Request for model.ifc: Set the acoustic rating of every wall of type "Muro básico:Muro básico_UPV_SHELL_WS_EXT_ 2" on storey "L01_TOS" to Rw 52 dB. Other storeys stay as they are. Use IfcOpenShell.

First a look at what the model holds.

```python
import ifcopenshell
import ifcopenshell.util.element

model = ifcopenshell.open("model.ifc")
print(model.schema)
storey = next(s for s in model.by_type("IfcBuildingStorey") if s.Name == "L01_TOS")
walls = [e for e in ifcopenshell.util.element.get_decomposition(storey) if e.is_a("IfcWall")]
seen = {}
for e in walls:
    element_type = ifcopenshell.util.element.get_type(e)
    key = (element_type.Name if element_type != e and element_type else None, ifcopenshell.util.element.get_pset(e, "Pset_WallCommon", "AcousticRating"))
    seen[key] = seen.get(key, 0) + 1
for (name, value), count in sorted(seen.items(), key=str):
    print(count, "x", name, "|", value)
```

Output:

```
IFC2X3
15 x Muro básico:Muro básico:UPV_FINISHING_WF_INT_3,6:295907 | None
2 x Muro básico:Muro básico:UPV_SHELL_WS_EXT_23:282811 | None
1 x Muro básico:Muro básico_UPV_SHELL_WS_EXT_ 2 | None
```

```python
import ifcopenshell
import ifcopenshell.api.pset
import ifcopenshell.util.element

model = ifcopenshell.open("model.ifc")

storey = next(s for s in model.by_type("IfcBuildingStorey") if s.Name == "L01_TOS")
walls = [e for e in ifcopenshell.util.element.get_decomposition(storey) if e.is_a("IfcWall")]

count = 0
for e in walls:
    element_type = ifcopenshell.util.element.get_type(e)
    if element_type in (None, e) or element_type.Name != "Muro básico:Muro básico_UPV_SHELL_WS_EXT_ 2":
        continue
    # add_pset returns the element's existing set when there is one.
    pset = ifcopenshell.api.pset.add_pset(model, product=e, name="Pset_WallCommon")
    ifcopenshell.api.pset.edit_pset(model, pset=pset, properties={"AcousticRating": "Rw 52 dB"})
    count += 1

print(count, "walls updated")

model.write("model-out.ifc")
```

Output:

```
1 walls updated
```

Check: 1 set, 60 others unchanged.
